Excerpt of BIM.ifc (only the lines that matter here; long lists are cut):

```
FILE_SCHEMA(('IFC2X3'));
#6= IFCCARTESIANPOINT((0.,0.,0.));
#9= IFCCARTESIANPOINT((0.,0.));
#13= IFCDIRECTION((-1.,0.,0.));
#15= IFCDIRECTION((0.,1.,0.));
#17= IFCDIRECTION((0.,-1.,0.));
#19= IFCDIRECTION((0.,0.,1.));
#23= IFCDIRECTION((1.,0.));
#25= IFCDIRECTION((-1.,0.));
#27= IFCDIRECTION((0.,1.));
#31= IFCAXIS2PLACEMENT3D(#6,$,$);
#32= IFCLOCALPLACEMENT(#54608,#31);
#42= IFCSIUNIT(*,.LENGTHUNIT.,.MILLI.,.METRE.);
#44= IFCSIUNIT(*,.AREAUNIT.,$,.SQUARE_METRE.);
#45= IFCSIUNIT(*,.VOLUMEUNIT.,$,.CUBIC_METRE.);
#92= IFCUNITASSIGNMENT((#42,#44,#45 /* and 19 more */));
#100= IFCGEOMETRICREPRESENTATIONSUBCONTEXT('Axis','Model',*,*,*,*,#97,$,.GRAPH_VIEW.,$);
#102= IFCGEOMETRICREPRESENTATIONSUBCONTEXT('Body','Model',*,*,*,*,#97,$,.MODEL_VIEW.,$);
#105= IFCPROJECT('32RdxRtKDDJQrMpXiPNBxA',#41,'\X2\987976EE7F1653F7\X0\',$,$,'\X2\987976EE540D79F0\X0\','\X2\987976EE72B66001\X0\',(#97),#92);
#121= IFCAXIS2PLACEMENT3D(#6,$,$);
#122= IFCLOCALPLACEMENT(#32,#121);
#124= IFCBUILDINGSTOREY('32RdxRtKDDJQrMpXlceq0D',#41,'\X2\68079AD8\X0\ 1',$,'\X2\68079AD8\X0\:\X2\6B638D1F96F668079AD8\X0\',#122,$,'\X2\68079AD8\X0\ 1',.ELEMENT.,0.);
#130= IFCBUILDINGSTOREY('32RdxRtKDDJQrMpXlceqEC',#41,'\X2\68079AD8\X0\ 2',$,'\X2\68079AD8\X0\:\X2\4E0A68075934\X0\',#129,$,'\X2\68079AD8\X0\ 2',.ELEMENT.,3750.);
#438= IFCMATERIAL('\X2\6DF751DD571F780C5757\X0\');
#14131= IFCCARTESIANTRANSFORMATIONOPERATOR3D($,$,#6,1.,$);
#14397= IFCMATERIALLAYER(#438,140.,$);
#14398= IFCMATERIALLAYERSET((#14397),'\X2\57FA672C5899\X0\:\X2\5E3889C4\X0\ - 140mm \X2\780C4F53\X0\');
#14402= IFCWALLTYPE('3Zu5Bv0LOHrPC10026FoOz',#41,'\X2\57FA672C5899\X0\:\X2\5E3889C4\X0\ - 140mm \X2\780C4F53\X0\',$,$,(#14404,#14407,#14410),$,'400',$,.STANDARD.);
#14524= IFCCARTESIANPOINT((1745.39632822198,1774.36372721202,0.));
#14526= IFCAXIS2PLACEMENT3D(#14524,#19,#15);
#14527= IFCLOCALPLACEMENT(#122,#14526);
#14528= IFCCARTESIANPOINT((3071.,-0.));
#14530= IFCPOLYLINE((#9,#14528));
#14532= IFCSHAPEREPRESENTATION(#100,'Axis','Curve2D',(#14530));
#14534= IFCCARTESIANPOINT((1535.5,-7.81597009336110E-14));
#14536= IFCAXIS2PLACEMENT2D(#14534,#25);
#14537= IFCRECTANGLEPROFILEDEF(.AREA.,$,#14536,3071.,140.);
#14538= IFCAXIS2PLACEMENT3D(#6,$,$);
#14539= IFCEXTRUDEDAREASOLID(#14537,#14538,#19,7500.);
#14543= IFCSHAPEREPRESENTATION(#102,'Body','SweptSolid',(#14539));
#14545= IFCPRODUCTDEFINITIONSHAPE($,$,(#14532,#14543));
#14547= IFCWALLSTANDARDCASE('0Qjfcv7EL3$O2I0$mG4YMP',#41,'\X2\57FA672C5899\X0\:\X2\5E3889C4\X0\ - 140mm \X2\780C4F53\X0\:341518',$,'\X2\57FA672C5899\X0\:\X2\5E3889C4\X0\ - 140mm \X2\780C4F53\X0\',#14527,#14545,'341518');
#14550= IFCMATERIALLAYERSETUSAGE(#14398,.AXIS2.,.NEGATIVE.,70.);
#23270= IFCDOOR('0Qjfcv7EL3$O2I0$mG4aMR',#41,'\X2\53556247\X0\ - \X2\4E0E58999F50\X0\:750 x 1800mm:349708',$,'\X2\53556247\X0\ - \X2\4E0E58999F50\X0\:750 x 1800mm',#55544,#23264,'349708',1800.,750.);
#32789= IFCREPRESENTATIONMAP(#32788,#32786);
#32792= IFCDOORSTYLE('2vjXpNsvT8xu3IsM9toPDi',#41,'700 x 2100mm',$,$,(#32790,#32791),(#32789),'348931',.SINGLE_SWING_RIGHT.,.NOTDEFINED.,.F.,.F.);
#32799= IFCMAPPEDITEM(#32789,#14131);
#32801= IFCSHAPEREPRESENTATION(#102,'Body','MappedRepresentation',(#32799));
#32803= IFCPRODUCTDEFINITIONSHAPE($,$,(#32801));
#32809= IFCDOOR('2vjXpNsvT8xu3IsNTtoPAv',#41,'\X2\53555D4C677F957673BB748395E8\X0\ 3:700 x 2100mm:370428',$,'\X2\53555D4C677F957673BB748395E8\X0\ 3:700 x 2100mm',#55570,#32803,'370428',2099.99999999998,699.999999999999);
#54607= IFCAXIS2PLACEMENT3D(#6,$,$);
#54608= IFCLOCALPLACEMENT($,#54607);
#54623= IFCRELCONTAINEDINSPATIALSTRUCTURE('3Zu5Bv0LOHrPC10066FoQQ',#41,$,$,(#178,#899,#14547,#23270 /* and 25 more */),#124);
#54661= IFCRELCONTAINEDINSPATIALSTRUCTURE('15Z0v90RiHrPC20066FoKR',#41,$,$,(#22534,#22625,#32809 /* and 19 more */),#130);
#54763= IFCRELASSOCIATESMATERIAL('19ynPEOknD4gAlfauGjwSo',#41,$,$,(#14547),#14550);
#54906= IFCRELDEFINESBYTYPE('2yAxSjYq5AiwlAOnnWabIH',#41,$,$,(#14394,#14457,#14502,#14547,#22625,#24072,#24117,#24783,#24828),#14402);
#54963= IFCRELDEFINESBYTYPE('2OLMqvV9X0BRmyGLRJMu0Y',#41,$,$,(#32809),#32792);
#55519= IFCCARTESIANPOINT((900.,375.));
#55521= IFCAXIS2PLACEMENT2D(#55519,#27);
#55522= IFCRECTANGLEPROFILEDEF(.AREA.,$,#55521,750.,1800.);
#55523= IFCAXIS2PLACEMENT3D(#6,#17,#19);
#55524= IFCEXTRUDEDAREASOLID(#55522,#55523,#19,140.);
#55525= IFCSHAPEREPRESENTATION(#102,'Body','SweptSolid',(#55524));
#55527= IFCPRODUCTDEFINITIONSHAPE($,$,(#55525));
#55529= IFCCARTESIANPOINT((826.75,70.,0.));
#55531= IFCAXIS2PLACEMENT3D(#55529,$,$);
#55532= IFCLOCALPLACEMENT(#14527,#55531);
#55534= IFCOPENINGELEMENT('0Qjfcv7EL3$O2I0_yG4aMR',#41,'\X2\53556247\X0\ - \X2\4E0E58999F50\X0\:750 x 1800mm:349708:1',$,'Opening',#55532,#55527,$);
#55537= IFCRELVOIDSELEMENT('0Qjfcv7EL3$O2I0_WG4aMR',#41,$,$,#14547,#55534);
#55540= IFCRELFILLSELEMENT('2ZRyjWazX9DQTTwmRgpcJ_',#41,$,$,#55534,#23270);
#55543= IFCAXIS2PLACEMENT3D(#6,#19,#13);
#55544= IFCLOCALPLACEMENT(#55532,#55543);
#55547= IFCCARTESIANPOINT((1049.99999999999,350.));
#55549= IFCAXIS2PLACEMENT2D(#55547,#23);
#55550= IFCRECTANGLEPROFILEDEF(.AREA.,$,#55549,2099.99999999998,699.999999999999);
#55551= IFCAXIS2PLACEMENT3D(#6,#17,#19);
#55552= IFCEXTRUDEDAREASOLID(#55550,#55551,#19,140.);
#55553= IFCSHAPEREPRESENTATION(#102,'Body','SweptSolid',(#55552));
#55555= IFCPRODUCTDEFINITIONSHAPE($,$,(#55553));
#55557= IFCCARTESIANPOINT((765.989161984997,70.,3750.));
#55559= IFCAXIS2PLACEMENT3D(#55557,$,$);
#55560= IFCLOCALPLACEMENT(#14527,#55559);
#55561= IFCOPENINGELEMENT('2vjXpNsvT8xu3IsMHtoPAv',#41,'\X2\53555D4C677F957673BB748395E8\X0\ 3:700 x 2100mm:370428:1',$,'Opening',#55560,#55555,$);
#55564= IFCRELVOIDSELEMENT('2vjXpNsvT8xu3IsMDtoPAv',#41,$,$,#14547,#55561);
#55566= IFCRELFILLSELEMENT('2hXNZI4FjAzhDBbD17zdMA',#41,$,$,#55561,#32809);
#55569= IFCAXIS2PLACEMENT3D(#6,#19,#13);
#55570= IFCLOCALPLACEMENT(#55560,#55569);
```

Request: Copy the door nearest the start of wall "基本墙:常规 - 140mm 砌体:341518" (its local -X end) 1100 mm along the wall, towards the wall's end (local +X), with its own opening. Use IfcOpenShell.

```python
import ifcopenshell
import ifcopenshell.api.feature
import ifcopenshell.api.geometry
import ifcopenshell.api.root
import ifcopenshell.geom
import ifcopenshell.util.element
import ifcopenshell.util.placement
import ifcopenshell.util.shape
import ifcopenshell.util.unit

model = ifcopenshell.open("BIM.ifc")
unit_scale = ifcopenshell.util.unit.calculate_unit_scale(model)
settings = ifcopenshell.geom.settings()


def volume(element):
    """Net volume in cubic metres, openings subtracted."""
    shape = ifcopenshell.geom.create_shape(settings, element)
    return ifcopenshell.util.shape.get_volume(shape.geometry)


def reuse_history(source, copy):
    """copy_class also copies each property set's owner history, people and application; keep the originals."""
    for rel in copy.IsDefinedBy:
        if rel.is_a("IfcRelDefinesByProperties") and (history := rel.RelatingPropertyDefinition.OwnerHistory):
            rel.RelatingPropertyDefinition.OwnerHistory = source.OwnerHistory
            ifcopenshell.util.element.remove_deep2(model, history)


door = model.by_id(32809)
opening = door.FillsVoids[0].RelatingOpeningElement
wall = opening.VoidsElements[0].RelatingBuildingElement
before = volume(wall)
shift = ifcopenshell.util.placement.get_local_placement(wall.ObjectPlacement)[:3, 0] * 1.1 / unit_scale

# copy_class copies the void relationship, type, container and properties, but no geometry.
new_opening = ifcopenshell.api.root.copy_class(model, product=opening)
new_opening.Representation = ifcopenshell.util.element.copy_deep(
    model, opening.Representation, exclude=["IfcGeometricRepresentationContext", "IfcRepresentationMap"]
)
new_opening.Name = "单嵌板镶玻璃门 3:700 x 2100mm"
new_door = ifcopenshell.api.root.copy_class(model, product=door)
new_door.Representation = ifcopenshell.util.element.copy_deep(
    model, door.Representation, exclude=["IfcGeometricRepresentationContext", "IfcRepresentationMap"]
)
new_door.Name = "单嵌板镶玻璃门 3:700 x 2100mm"
new_door.Tag = None
reuse_history(door, new_door)
fills = ifcopenshell.api.feature.add_filling(model, opening=new_opening, element=new_door)
fills.OwnerHistory = new_door.OwnerHistory  # required in IFC2X3

for old, new in ((opening, new_opening), (door, new_door)):
    matrix = ifcopenshell.util.placement.get_local_placement(old.ObjectPlacement)
    matrix[:3, 3] += shift
    ifcopenshell.api.geometry.edit_object_placement(model, product=new, matrix=matrix, is_si=False)

after = volume(wall)

print(f"wall volume {before:.3f} -> {after:.3f} m3")

model.write("BIM_edited.ifc")
```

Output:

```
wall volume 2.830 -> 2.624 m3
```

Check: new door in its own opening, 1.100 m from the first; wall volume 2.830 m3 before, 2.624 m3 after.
